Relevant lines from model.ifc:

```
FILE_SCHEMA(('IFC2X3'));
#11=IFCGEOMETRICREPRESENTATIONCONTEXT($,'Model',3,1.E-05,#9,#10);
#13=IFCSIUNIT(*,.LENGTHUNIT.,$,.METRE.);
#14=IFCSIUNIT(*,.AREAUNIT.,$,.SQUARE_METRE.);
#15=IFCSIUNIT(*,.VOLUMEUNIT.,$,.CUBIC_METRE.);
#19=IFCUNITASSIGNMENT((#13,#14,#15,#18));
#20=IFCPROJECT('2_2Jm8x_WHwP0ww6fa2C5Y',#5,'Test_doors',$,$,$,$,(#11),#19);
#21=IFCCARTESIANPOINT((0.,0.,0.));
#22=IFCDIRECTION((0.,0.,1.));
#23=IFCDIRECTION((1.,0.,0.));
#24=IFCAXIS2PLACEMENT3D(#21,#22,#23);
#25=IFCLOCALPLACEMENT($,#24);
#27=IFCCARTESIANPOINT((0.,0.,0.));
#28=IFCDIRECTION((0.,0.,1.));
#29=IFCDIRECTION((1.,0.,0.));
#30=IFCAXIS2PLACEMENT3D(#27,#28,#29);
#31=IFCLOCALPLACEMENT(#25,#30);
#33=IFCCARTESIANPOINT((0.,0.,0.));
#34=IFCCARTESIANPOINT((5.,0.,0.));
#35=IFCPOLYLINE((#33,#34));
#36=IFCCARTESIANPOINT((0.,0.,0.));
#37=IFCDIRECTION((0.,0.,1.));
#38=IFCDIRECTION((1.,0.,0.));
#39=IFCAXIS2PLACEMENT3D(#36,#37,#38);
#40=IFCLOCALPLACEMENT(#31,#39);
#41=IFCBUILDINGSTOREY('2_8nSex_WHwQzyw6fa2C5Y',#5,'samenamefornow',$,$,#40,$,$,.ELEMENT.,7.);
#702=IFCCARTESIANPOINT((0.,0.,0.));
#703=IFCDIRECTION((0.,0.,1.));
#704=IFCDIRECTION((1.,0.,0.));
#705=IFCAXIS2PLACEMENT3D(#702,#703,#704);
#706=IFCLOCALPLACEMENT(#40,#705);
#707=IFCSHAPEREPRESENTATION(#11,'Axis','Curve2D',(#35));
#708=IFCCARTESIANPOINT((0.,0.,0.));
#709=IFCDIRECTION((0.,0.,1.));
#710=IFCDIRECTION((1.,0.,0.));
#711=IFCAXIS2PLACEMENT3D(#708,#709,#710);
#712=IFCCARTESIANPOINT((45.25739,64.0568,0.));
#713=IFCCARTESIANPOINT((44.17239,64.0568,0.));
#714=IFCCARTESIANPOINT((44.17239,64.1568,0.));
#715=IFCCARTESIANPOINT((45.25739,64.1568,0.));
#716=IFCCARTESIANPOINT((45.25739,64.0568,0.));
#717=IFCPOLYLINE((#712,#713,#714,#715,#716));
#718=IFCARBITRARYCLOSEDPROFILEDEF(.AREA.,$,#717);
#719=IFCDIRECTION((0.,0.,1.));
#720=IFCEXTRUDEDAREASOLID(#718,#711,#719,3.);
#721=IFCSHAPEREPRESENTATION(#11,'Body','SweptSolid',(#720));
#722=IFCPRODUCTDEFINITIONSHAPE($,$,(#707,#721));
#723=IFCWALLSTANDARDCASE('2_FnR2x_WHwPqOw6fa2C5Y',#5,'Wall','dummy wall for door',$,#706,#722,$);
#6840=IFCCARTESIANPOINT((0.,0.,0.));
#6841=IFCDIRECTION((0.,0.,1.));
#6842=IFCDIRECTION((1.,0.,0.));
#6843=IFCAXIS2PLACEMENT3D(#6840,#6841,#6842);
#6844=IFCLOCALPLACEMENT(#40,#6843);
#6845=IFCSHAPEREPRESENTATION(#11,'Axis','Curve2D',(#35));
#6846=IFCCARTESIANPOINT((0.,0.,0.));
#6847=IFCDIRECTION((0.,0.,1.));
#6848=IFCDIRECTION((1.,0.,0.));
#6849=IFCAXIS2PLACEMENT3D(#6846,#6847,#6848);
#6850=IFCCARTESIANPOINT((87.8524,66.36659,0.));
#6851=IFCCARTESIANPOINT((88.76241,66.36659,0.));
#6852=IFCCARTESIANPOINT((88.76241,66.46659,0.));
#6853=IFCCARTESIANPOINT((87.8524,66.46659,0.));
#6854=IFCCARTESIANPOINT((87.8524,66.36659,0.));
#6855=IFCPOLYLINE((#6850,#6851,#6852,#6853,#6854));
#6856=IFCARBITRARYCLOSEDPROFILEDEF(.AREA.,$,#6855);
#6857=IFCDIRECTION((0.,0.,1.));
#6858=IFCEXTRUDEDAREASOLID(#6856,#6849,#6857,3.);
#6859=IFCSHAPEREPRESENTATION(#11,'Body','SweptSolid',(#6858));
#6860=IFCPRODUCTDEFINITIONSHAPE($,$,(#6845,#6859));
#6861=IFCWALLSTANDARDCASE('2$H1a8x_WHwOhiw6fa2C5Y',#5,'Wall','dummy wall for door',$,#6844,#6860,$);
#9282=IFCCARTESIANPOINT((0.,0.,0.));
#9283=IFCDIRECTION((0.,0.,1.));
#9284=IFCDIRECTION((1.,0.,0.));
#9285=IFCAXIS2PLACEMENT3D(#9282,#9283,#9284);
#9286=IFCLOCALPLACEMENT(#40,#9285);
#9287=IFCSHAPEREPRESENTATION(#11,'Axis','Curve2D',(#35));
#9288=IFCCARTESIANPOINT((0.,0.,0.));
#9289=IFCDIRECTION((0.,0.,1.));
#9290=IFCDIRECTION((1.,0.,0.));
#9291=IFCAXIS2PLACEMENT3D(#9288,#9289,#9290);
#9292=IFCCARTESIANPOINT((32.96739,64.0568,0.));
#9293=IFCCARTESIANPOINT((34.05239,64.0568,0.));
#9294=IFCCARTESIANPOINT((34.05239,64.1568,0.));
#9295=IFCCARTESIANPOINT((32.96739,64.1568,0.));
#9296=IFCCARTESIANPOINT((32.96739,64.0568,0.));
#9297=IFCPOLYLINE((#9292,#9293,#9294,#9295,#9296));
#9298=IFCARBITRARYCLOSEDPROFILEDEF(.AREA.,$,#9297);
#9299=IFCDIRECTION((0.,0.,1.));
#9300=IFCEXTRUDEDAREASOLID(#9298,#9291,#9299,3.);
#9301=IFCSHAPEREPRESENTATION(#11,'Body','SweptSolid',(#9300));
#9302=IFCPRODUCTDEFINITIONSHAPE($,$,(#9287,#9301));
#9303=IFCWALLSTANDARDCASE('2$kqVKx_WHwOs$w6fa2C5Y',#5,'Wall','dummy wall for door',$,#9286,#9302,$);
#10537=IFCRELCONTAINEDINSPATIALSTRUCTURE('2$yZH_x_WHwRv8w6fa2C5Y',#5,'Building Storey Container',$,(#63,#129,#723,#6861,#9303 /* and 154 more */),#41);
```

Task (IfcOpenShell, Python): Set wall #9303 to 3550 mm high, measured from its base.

```python
import ifcopenshell
import ifcopenshell.geom
import ifcopenshell.util.shape
import ifcopenshell.util.unit

model = ifcopenshell.open("model.ifc")
unit_scale = ifcopenshell.util.unit.calculate_unit_scale(model)
settings = ifcopenshell.geom.settings()


def volume(element):
    """Net volume in cubic metres, openings subtracted."""
    shape = ifcopenshell.geom.create_shape(settings, element)
    return ifcopenshell.util.shape.get_volume(shape.geometry)


wall = model.by_guid("2$kqVKx_WHwOs$w6fa2C5Y")
before = volume(wall)

body = next(r for r in wall.Representation.Representations if r.RepresentationIdentifier == "Body")
solid = body.Items[0]
old_height = solid.Depth
solid.Depth = 3.55 / unit_scale
after = volume(wall)

print(f"height {old_height:g} -> {solid.Depth:g}, volume {before:.3f} -> {after:.3f} m3")

model.write("model_updated.ifc")
```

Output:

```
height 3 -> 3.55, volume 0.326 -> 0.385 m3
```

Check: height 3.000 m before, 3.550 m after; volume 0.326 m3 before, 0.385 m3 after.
